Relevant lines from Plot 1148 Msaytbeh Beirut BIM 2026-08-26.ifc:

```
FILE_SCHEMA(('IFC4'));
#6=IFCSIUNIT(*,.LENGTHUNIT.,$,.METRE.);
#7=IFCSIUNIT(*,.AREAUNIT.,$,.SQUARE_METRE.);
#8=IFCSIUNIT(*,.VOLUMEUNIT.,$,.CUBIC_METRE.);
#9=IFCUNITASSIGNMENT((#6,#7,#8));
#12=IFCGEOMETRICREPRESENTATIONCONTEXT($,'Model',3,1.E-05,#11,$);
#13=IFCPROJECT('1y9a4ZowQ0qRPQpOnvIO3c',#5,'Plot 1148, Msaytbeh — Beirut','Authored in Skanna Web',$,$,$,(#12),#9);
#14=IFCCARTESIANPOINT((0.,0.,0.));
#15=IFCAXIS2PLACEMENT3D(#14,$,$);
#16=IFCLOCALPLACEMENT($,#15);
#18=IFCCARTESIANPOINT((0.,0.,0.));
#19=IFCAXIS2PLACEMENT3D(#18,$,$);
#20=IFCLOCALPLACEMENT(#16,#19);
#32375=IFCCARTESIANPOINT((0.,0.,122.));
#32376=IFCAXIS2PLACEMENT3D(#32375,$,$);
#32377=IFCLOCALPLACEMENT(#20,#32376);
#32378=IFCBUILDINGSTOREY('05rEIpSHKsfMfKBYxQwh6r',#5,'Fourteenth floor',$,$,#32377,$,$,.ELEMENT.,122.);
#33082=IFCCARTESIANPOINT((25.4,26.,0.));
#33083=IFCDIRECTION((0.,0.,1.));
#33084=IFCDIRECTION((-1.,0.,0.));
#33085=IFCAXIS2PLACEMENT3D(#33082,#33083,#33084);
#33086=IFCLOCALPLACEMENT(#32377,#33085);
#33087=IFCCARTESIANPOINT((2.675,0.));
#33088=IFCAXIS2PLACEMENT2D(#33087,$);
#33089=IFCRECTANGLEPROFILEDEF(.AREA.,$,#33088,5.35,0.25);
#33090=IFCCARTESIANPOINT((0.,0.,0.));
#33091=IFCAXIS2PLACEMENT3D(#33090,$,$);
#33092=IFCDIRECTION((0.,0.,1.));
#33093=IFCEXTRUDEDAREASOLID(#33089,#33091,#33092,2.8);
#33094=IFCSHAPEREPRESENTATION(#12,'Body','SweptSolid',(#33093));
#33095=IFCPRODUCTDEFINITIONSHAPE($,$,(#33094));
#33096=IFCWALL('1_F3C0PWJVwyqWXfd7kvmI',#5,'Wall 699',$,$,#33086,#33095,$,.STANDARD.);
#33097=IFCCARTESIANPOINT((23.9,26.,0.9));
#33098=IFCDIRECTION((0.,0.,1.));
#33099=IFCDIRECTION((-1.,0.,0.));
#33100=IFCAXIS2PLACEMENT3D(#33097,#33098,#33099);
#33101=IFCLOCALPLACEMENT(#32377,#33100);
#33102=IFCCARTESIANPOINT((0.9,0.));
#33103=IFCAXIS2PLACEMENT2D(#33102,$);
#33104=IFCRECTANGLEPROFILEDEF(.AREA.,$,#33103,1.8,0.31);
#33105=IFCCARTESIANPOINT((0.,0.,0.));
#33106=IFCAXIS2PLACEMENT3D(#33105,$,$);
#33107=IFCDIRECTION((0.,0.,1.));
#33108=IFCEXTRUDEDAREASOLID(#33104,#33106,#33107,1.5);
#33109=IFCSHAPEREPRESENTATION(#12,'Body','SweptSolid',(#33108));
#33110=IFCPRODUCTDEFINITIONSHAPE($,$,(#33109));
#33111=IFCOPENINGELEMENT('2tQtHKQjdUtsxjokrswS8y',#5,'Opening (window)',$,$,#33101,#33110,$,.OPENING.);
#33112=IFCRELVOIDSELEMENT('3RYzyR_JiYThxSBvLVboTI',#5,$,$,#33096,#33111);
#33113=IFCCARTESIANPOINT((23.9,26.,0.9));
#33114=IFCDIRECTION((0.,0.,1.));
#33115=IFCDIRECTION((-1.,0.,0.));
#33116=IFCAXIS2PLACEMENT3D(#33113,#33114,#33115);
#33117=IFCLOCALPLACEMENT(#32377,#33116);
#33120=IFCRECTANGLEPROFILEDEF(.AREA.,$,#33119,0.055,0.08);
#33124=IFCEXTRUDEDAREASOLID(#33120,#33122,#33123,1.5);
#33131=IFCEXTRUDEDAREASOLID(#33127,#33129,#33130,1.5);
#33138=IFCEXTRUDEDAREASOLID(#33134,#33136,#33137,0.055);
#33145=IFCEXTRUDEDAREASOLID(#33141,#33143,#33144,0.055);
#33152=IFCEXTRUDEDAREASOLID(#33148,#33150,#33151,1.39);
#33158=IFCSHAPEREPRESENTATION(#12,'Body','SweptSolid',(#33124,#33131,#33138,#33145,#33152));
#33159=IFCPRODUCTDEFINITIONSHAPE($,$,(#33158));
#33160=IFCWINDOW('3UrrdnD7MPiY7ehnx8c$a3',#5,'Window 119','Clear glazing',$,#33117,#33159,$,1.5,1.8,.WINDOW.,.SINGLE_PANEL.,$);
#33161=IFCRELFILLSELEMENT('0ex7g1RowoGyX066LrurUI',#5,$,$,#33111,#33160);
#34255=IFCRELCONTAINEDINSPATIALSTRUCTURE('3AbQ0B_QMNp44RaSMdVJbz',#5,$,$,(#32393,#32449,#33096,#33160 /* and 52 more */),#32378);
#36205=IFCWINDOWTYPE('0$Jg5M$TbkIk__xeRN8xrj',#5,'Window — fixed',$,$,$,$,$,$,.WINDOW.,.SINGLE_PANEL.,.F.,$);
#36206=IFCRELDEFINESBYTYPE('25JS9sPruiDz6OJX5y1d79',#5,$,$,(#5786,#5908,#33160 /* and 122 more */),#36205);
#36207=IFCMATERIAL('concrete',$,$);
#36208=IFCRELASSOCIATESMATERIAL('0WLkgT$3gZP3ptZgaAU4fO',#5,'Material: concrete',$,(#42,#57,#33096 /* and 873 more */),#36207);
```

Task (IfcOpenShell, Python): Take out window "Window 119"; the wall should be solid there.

```python
import ifcopenshell
import ifcopenshell.api.feature
import ifcopenshell.api.root
import ifcopenshell.geom
import ifcopenshell.util.shape

model = ifcopenshell.open("Plot 1148 Msaytbeh Beirut BIM 2026-08-26.ifc")
settings = ifcopenshell.geom.settings()


def volume(element):
    """Net volume in cubic metres, openings subtracted."""
    shape = ifcopenshell.geom.create_shape(settings, element)
    return ifcopenshell.util.shape.get_volume(shape.geometry)


window = model.by_guid("3UrrdnD7MPiY7ehnx8c$a3")
opening = window.FillsVoids[0].RelatingOpeningElement
wall = opening.VoidsElements[0].RelatingBuildingElement
before = volume(wall)

ifcopenshell.api.root.remove_product(model, product=window)
ifcopenshell.api.feature.remove_feature(model, feature=opening)

after = volume(wall)

print(f"wall volume {before:.3f} -> {after:.3f} m3")

model.write("Plot 1148 Msaytbeh Beirut BIM 2026-08-26_v2.ifc")
```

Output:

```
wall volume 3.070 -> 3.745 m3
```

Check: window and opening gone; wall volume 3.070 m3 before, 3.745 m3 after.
